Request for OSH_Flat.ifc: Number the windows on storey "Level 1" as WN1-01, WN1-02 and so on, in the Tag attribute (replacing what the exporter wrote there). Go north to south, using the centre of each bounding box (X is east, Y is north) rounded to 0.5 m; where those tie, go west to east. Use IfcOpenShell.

First a look at what the model holds.

```python
import ifcopenshell
import ifcopenshell.util.element
import ifcopenshell.util.placement

model = ifcopenshell.open("OSH_Flat.ifc")
print(model.schema)
storey = next(s for s in model.by_type("IfcBuildingStorey") if s.Name == "Level 1")
windows = [e for e in ifcopenshell.util.element.get_decomposition(storey) if e.is_a("IfcWindow")]
for e in sorted(windows, key=lambda e: e.id()):
    origin = ifcopenshell.util.placement.get_local_placement(e.ObjectPlacement)[:3, 3]
    print(e.id(), e.Tag, e.Name, origin.round(2) + 0.0, sep=" | ")
```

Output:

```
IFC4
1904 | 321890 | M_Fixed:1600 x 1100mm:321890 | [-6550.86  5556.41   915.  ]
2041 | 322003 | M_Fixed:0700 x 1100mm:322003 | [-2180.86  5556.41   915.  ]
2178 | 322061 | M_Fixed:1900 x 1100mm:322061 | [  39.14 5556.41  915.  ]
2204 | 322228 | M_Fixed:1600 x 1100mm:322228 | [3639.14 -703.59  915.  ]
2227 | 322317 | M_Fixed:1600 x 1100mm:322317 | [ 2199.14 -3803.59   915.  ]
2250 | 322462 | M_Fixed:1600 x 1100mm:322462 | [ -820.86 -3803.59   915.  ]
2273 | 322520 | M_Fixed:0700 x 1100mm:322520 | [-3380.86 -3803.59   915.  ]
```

```python
import ifcopenshell
import ifcopenshell.geom
import ifcopenshell.util.element
import ifcopenshell.util.shape

model = ifcopenshell.open("OSH_Flat.ifc")
settings = ifcopenshell.geom.settings()
settings.set("use-world-coords", True)


def centre(element):
    shape = ifcopenshell.geom.create_shape(settings, element)
    return ifcopenshell.util.shape.get_bbox_centroid(shape.geometry)


storey = next(s for s in model.by_type("IfcBuildingStorey") if s.Name == "Level 1")
windows = [e for e in ifcopenshell.util.element.get_decomposition(storey) if e.is_a("IfcWindow")]

# Insertion points can sit at a corner or the storey origin, so sort by the geometry (in metres).
centres = {e: centre(e) for e in windows}
windows.sort(key=lambda e: (-round(centres[e][1] / 0.5), centres[e][0]))

for i, e in enumerate(windows, start=1):
    number = f"WN1-{i:02d}"
    e.Tag = number
    print(e.id(), number)

model.write("OSH_Flat-out.ifc")
```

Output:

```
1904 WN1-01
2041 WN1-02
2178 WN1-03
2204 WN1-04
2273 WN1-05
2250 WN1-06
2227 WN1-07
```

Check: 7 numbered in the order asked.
